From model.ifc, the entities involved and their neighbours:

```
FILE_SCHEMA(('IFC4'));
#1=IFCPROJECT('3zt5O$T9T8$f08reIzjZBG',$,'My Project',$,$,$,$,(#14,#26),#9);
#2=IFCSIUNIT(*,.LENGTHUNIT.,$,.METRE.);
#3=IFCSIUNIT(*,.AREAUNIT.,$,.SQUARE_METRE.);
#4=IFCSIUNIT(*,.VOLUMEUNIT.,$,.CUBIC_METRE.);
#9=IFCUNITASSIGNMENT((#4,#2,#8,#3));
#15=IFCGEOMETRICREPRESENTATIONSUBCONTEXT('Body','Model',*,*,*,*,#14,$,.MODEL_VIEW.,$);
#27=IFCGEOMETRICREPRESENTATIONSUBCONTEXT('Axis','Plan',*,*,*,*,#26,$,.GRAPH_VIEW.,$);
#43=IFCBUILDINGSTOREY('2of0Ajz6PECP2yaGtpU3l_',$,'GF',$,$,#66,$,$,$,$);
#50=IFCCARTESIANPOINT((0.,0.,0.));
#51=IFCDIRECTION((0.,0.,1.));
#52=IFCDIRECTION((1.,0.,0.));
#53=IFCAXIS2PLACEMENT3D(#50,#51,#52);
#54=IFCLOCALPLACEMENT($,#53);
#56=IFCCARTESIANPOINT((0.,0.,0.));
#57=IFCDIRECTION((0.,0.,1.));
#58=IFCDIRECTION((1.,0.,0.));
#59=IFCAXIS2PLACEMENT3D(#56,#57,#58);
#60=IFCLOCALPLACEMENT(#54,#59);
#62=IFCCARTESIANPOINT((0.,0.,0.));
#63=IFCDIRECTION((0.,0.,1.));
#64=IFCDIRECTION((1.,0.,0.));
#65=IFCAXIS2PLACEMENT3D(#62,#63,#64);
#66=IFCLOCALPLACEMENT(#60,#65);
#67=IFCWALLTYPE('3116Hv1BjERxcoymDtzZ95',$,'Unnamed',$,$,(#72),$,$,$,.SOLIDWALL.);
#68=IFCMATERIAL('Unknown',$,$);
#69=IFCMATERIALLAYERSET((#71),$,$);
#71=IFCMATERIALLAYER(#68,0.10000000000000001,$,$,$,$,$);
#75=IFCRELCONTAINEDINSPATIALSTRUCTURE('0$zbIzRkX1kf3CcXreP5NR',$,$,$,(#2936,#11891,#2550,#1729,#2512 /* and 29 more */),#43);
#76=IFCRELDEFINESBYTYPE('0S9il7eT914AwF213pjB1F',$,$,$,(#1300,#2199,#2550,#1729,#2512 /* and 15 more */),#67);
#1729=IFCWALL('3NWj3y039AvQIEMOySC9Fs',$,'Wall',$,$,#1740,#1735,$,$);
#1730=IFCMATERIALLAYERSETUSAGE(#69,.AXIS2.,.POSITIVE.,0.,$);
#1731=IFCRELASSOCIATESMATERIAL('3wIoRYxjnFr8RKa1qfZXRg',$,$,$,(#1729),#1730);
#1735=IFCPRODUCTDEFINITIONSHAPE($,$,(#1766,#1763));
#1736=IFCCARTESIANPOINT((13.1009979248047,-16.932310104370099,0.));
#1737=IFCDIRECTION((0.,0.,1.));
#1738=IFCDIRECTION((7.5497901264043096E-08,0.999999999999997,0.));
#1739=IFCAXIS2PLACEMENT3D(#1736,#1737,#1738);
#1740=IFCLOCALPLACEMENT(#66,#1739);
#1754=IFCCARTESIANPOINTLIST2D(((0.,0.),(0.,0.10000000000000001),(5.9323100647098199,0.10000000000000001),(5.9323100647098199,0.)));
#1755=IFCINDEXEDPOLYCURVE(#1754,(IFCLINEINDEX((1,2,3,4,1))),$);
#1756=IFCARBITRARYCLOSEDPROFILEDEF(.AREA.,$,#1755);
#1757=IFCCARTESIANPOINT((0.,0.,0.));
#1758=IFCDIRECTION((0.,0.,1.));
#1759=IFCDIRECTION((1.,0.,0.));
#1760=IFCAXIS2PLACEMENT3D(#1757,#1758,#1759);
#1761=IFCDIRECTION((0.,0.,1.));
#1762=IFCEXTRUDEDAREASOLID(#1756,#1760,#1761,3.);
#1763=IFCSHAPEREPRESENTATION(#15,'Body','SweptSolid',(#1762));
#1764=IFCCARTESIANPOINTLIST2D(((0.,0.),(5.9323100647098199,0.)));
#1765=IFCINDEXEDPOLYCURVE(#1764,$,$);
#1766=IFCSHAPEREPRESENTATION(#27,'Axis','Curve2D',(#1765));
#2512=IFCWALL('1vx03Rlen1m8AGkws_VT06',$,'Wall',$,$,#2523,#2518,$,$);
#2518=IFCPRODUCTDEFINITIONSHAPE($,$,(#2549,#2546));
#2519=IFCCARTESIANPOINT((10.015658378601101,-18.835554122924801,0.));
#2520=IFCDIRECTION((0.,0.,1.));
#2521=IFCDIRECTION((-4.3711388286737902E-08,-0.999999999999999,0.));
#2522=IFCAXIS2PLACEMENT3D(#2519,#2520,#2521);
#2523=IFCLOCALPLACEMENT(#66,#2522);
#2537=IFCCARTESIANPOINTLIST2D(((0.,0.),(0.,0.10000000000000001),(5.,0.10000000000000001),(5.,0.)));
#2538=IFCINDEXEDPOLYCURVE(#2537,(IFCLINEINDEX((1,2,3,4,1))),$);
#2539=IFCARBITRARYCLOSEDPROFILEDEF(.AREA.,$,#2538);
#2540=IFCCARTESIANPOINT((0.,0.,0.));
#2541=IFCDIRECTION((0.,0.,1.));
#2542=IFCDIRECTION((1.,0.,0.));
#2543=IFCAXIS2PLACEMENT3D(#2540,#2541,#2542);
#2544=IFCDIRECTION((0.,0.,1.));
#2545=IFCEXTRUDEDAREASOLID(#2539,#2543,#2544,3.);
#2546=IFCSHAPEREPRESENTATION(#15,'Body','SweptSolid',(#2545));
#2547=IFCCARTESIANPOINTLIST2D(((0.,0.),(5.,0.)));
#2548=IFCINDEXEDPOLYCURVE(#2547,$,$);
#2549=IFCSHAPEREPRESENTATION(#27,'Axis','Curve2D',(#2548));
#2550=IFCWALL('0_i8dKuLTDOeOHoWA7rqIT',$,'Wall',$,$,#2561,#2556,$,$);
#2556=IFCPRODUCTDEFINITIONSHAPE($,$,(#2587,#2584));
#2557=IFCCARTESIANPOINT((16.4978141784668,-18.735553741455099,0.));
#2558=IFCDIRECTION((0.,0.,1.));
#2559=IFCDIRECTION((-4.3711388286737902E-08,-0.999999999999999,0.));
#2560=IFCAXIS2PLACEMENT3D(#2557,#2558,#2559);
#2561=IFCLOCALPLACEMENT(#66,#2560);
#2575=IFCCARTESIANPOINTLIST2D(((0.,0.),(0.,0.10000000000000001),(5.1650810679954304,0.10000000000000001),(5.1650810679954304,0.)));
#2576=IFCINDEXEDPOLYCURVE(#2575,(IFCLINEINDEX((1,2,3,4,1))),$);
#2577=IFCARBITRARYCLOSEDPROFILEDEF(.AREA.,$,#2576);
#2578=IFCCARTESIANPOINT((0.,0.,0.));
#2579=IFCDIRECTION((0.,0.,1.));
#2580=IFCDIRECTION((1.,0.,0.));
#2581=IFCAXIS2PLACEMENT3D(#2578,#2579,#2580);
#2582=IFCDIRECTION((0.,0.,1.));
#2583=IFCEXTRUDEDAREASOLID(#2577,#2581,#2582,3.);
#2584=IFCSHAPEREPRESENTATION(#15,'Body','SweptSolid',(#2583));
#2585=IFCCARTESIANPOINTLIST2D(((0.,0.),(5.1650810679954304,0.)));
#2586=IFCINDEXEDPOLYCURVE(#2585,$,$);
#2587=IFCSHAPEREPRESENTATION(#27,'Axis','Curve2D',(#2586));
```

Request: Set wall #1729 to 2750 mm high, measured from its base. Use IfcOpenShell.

```python
import ifcopenshell
import ifcopenshell.geom
import ifcopenshell.util.representation
import ifcopenshell.util.shape

model = ifcopenshell.open("model.ifc")
settings = ifcopenshell.geom.settings()


def volume(element):
    """Net volume in cubic metres, openings subtracted."""
    shape = ifcopenshell.geom.create_shape(settings, element)
    return ifcopenshell.util.shape.get_volume(shape.geometry)


wall = model.by_guid("3NWj3y039AvQIEMOySC9Fs")
before = volume(wall)

body = ifcopenshell.util.representation.get_representation(wall, "Model", "Body")
solid = body.Items[0]
old_height = solid.Depth
solid.Depth = 2.75
after = volume(wall)

print(f"height {old_height:g} -> {solid.Depth:g}, volume {before:.3f} -> {after:.3f} m3")

model.write("model_edited.ifc")
```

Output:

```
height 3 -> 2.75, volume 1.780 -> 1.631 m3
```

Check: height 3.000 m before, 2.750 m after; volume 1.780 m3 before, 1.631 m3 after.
